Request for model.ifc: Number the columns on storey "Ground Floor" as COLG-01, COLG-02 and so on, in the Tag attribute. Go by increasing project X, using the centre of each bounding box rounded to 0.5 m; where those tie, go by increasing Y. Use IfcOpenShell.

First a look at what the model holds.

```python
import ifcopenshell
import ifcopenshell.util.element
import ifcopenshell.util.placement

model = ifcopenshell.open("model.ifc")
print(model.schema)
storey = next(s for s in model.by_type("IfcBuildingStorey") if s.Name == "Ground Floor")
columns = [e for e in ifcopenshell.util.element.get_decomposition(storey) if e.is_a("IfcColumn")]
for e in sorted(columns, key=lambda e: e.id()):
    origin = ifcopenshell.util.placement.get_local_placement(e.ObjectPlacement)[:3, 3]
    print(e.id(), e.Tag, e.Name, origin.round(2) + 0.0, sep=" | ")
```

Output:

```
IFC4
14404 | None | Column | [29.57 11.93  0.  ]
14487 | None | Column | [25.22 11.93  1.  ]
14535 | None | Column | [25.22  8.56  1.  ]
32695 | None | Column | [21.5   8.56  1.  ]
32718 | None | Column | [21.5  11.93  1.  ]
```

```python
import ifcopenshell
import ifcopenshell.geom
import ifcopenshell.util.element
import ifcopenshell.util.shape

model = ifcopenshell.open("model.ifc")
settings = ifcopenshell.geom.settings()
settings.set("use-world-coords", True)


def centre(element):
    shape = ifcopenshell.geom.create_shape(settings, element)
    return ifcopenshell.util.shape.get_bbox_centroid(shape.geometry)


storey = next(s for s in model.by_type("IfcBuildingStorey") if s.Name == "Ground Floor")
columns = [e for e in ifcopenshell.util.element.get_decomposition(storey) if e.is_a("IfcColumn")]

# Insertion points can sit at a corner or the storey origin, so sort by the geometry (in metres).
centres = {e: centre(e) for e in columns}
columns.sort(key=lambda e: (round(centres[e][0] / 0.5), centres[e][1]))

for i, e in enumerate(columns, start=1):
    number = f"COLG-{i:02d}"
    e.Tag = number
    print(e.id(), number)

model.write("model_rev.ifc")
```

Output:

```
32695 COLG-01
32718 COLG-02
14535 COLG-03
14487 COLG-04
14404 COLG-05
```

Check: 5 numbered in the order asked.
